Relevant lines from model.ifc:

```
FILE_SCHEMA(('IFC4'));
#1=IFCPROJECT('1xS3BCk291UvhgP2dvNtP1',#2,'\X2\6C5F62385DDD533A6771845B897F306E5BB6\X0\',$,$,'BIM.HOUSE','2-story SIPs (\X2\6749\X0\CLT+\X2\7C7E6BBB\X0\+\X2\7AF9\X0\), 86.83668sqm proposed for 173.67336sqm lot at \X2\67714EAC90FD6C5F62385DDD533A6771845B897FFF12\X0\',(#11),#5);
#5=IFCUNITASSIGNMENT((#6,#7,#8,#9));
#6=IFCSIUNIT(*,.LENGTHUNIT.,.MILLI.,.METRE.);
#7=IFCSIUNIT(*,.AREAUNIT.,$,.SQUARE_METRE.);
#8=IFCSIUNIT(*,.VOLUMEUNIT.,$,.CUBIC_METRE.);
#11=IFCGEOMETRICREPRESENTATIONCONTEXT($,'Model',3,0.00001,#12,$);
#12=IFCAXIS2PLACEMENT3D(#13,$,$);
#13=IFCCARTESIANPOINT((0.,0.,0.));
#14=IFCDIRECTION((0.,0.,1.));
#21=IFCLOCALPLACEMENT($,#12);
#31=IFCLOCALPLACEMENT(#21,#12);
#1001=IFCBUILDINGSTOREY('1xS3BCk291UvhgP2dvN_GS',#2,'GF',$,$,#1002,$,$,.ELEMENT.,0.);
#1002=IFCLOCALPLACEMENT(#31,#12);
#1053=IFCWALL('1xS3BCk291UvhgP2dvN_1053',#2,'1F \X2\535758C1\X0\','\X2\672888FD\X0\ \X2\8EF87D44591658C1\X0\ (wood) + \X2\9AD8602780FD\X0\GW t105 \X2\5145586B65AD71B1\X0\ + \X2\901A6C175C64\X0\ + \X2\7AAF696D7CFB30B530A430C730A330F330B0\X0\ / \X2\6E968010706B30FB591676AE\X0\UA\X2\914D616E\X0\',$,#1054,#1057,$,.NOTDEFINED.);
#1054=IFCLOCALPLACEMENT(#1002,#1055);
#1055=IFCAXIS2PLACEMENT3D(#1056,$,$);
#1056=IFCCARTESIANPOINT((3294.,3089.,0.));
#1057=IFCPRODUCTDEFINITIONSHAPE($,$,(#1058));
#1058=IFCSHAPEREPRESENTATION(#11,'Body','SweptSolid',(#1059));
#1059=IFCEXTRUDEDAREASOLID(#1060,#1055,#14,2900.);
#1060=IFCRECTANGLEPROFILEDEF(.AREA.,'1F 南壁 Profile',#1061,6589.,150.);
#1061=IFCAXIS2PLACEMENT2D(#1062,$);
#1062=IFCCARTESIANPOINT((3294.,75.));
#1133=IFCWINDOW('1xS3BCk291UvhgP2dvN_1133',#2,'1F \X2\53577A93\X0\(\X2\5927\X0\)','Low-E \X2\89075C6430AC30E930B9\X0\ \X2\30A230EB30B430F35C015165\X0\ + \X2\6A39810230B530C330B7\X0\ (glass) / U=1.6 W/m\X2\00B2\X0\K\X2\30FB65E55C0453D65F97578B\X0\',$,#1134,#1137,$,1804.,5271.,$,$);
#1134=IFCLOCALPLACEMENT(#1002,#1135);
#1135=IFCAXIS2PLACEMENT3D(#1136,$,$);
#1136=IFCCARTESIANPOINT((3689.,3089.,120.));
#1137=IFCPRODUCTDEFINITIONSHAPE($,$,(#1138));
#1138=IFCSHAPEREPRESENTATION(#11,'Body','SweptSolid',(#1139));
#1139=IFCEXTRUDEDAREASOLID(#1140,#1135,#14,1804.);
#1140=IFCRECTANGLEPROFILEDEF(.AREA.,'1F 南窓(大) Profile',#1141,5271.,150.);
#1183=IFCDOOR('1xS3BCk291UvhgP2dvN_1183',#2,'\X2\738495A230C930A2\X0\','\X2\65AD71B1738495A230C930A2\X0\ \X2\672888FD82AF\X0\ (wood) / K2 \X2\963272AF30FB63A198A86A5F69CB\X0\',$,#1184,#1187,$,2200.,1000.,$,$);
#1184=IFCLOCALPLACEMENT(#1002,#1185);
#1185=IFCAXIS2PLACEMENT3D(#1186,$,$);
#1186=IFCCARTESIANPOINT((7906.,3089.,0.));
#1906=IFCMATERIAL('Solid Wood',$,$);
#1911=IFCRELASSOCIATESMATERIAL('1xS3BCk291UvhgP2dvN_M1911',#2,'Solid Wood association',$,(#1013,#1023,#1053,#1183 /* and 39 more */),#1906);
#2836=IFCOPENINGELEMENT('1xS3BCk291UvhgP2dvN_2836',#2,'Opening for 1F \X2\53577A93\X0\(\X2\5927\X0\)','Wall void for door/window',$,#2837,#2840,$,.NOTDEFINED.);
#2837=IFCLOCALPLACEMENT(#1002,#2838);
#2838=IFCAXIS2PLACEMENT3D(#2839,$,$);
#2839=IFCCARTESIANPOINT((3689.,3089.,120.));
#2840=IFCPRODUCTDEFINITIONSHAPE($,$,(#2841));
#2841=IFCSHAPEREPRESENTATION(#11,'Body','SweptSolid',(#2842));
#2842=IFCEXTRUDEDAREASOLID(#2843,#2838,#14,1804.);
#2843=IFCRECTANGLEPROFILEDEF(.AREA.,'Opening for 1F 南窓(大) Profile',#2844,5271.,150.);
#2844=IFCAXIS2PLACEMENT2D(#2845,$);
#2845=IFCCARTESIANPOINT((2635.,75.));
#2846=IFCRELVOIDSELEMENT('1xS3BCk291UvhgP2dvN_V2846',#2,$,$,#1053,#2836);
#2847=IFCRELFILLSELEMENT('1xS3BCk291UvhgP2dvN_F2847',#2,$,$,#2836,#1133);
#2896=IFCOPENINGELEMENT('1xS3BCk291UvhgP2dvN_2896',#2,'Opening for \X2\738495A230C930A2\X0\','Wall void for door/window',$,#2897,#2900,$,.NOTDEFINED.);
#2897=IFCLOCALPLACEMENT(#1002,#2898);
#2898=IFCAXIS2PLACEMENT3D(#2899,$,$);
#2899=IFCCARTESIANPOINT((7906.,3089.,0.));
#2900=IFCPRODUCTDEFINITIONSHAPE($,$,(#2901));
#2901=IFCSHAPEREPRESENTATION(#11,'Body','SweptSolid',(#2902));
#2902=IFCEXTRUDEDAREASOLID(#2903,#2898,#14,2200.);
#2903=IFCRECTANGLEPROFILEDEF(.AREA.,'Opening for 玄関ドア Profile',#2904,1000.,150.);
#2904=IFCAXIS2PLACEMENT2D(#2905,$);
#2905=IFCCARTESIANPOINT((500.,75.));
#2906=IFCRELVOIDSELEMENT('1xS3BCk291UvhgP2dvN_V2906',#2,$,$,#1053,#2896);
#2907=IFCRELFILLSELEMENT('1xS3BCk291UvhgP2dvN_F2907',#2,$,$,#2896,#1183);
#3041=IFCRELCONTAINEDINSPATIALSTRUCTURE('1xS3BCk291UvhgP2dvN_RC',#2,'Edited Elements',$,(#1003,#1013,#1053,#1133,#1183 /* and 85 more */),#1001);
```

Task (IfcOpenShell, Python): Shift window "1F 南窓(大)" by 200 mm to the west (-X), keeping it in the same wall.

```python
import ifcopenshell
import ifcopenshell.api.geometry
import ifcopenshell.util.placement
import ifcopenshell.util.unit

model = ifcopenshell.open("model.ifc")
unit_scale = ifcopenshell.util.unit.calculate_unit_scale(model)

window = model.by_guid("1xS3BCk291UvhgP2dvN_1133")
opening = window.FillsVoids[0].RelatingOpeningElement
wall = opening.VoidsElements[0].RelatingBuildingElement

wall_matrix = ifcopenshell.util.placement.get_local_placement(wall.ObjectPlacement)
shift = wall_matrix[:3, 0] * -0.2 / unit_scale
before = ifcopenshell.util.placement.get_local_placement(window.ObjectPlacement)[:3, 3].copy()

# The window is not placed relative to its opening, so move both.
for product in (opening, window):
    matrix = ifcopenshell.util.placement.get_local_placement(product.ObjectPlacement)
    matrix[:3, 3] += shift
    ifcopenshell.api.geometry.edit_object_placement(model, product=product, matrix=matrix, is_si=False)

after = ifcopenshell.util.placement.get_local_placement(window.ObjectPlacement)[:3, 3]
print("window moved by", (after - before).round(3) + 0.0)

model.write("model_rev.ifc")
```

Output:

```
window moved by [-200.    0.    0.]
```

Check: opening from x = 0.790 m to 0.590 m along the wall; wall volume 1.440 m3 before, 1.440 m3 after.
